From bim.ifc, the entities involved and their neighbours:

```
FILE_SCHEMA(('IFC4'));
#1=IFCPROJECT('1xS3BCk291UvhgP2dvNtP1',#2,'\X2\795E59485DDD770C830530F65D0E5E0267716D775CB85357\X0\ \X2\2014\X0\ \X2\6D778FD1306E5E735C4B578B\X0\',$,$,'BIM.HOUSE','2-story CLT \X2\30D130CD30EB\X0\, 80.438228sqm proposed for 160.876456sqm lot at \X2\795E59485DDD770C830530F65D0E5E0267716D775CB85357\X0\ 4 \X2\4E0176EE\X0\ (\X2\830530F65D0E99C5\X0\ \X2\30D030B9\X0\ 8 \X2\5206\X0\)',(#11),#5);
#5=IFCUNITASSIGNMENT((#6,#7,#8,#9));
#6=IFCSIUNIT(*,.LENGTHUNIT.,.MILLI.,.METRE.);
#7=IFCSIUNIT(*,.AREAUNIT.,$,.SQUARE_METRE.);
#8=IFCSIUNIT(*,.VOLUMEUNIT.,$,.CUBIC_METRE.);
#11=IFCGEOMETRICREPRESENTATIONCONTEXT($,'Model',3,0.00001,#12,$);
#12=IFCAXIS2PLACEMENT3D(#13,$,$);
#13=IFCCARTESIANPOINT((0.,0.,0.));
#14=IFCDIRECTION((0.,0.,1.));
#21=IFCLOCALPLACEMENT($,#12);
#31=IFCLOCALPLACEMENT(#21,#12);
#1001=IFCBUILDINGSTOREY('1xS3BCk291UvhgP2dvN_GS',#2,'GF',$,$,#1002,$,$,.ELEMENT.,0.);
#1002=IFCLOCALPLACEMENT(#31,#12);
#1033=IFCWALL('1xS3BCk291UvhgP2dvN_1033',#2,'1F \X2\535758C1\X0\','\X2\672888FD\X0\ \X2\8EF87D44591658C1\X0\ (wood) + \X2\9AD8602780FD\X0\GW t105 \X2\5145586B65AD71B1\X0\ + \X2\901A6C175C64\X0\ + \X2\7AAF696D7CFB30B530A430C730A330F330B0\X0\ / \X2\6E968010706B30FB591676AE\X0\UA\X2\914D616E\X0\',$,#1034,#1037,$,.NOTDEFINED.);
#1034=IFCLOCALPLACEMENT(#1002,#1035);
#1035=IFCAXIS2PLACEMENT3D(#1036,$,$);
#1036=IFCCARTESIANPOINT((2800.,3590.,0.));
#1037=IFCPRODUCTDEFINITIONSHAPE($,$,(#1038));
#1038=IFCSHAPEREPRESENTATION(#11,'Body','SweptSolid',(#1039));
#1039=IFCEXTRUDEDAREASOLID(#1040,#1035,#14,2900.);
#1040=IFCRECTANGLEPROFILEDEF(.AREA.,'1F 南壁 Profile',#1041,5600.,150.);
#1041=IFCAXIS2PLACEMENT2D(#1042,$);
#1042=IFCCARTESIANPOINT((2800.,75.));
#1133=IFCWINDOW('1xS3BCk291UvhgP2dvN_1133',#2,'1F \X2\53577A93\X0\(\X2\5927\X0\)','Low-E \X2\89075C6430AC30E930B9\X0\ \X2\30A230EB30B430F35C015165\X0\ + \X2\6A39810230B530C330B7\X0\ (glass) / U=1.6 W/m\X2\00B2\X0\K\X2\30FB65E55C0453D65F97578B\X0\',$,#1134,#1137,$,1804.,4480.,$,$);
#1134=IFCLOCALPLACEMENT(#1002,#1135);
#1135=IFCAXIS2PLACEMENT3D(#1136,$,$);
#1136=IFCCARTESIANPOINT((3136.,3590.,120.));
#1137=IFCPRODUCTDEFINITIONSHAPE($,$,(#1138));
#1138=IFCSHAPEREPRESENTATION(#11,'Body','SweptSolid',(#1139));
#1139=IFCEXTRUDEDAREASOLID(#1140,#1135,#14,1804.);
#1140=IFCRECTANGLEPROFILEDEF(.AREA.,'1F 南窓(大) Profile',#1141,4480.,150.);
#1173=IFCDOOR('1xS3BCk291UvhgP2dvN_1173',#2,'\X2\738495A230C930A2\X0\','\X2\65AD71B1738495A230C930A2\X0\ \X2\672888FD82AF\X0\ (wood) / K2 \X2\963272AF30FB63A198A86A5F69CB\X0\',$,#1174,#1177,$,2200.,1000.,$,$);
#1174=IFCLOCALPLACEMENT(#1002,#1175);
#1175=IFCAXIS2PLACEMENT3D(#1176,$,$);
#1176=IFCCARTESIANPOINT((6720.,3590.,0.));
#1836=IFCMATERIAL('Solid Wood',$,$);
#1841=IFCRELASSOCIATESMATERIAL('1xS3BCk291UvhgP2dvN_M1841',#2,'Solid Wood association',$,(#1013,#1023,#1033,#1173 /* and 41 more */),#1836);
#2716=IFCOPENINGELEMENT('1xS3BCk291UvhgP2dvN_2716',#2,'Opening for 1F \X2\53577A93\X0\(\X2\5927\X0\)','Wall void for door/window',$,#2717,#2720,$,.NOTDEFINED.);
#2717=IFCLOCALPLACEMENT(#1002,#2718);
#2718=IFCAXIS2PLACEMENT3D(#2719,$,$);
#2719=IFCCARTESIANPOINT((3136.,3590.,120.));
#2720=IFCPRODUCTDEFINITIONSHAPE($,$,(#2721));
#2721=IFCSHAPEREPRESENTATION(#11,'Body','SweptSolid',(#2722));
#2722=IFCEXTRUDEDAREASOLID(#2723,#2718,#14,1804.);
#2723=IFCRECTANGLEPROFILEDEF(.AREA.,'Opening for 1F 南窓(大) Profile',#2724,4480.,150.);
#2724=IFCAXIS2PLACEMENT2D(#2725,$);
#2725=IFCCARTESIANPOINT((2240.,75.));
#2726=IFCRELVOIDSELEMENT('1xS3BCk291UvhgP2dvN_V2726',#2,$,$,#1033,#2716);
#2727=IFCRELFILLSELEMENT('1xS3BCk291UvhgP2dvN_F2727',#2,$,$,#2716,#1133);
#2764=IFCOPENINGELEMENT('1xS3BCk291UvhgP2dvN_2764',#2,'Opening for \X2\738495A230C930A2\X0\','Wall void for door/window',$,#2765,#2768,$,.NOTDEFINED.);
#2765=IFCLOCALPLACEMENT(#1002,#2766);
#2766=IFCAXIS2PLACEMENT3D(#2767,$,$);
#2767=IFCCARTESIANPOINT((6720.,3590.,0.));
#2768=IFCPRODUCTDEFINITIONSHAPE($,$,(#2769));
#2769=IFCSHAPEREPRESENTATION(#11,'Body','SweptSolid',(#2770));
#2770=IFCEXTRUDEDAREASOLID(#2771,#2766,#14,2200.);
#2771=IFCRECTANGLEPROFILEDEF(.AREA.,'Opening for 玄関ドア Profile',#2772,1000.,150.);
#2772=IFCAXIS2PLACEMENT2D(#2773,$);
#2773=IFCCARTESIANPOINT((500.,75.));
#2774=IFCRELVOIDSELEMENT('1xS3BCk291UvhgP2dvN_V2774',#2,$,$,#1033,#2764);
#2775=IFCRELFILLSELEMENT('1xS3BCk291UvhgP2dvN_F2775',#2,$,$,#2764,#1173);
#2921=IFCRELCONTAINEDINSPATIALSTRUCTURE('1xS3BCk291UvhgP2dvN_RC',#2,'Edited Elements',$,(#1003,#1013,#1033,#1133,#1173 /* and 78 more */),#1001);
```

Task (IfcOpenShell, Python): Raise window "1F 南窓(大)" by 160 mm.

```python
import numpy as np
import ifcopenshell
import ifcopenshell.api.geometry
import ifcopenshell.util.placement
import ifcopenshell.util.unit

model = ifcopenshell.open("bim.ifc")
unit_scale = ifcopenshell.util.unit.calculate_unit_scale(model)

window = model.by_id(1133)
opening = window.FillsVoids[0].RelatingOpeningElement
dz = 160.0

shift = np.array([0.0, 0.0, dz])
# The window is not placed relative to its opening, so move both.
for product in (opening, window):
    matrix = ifcopenshell.util.placement.get_local_placement(product.ObjectPlacement)
    matrix[:3, 3] += shift
    ifcopenshell.api.geometry.edit_object_placement(model, product=product, matrix=matrix, is_si=False)

print(f"moved by {dz * unit_scale:+.3f} m")

model.write("bim_v2.ifc")
```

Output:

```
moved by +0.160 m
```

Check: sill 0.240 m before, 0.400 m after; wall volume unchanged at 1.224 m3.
